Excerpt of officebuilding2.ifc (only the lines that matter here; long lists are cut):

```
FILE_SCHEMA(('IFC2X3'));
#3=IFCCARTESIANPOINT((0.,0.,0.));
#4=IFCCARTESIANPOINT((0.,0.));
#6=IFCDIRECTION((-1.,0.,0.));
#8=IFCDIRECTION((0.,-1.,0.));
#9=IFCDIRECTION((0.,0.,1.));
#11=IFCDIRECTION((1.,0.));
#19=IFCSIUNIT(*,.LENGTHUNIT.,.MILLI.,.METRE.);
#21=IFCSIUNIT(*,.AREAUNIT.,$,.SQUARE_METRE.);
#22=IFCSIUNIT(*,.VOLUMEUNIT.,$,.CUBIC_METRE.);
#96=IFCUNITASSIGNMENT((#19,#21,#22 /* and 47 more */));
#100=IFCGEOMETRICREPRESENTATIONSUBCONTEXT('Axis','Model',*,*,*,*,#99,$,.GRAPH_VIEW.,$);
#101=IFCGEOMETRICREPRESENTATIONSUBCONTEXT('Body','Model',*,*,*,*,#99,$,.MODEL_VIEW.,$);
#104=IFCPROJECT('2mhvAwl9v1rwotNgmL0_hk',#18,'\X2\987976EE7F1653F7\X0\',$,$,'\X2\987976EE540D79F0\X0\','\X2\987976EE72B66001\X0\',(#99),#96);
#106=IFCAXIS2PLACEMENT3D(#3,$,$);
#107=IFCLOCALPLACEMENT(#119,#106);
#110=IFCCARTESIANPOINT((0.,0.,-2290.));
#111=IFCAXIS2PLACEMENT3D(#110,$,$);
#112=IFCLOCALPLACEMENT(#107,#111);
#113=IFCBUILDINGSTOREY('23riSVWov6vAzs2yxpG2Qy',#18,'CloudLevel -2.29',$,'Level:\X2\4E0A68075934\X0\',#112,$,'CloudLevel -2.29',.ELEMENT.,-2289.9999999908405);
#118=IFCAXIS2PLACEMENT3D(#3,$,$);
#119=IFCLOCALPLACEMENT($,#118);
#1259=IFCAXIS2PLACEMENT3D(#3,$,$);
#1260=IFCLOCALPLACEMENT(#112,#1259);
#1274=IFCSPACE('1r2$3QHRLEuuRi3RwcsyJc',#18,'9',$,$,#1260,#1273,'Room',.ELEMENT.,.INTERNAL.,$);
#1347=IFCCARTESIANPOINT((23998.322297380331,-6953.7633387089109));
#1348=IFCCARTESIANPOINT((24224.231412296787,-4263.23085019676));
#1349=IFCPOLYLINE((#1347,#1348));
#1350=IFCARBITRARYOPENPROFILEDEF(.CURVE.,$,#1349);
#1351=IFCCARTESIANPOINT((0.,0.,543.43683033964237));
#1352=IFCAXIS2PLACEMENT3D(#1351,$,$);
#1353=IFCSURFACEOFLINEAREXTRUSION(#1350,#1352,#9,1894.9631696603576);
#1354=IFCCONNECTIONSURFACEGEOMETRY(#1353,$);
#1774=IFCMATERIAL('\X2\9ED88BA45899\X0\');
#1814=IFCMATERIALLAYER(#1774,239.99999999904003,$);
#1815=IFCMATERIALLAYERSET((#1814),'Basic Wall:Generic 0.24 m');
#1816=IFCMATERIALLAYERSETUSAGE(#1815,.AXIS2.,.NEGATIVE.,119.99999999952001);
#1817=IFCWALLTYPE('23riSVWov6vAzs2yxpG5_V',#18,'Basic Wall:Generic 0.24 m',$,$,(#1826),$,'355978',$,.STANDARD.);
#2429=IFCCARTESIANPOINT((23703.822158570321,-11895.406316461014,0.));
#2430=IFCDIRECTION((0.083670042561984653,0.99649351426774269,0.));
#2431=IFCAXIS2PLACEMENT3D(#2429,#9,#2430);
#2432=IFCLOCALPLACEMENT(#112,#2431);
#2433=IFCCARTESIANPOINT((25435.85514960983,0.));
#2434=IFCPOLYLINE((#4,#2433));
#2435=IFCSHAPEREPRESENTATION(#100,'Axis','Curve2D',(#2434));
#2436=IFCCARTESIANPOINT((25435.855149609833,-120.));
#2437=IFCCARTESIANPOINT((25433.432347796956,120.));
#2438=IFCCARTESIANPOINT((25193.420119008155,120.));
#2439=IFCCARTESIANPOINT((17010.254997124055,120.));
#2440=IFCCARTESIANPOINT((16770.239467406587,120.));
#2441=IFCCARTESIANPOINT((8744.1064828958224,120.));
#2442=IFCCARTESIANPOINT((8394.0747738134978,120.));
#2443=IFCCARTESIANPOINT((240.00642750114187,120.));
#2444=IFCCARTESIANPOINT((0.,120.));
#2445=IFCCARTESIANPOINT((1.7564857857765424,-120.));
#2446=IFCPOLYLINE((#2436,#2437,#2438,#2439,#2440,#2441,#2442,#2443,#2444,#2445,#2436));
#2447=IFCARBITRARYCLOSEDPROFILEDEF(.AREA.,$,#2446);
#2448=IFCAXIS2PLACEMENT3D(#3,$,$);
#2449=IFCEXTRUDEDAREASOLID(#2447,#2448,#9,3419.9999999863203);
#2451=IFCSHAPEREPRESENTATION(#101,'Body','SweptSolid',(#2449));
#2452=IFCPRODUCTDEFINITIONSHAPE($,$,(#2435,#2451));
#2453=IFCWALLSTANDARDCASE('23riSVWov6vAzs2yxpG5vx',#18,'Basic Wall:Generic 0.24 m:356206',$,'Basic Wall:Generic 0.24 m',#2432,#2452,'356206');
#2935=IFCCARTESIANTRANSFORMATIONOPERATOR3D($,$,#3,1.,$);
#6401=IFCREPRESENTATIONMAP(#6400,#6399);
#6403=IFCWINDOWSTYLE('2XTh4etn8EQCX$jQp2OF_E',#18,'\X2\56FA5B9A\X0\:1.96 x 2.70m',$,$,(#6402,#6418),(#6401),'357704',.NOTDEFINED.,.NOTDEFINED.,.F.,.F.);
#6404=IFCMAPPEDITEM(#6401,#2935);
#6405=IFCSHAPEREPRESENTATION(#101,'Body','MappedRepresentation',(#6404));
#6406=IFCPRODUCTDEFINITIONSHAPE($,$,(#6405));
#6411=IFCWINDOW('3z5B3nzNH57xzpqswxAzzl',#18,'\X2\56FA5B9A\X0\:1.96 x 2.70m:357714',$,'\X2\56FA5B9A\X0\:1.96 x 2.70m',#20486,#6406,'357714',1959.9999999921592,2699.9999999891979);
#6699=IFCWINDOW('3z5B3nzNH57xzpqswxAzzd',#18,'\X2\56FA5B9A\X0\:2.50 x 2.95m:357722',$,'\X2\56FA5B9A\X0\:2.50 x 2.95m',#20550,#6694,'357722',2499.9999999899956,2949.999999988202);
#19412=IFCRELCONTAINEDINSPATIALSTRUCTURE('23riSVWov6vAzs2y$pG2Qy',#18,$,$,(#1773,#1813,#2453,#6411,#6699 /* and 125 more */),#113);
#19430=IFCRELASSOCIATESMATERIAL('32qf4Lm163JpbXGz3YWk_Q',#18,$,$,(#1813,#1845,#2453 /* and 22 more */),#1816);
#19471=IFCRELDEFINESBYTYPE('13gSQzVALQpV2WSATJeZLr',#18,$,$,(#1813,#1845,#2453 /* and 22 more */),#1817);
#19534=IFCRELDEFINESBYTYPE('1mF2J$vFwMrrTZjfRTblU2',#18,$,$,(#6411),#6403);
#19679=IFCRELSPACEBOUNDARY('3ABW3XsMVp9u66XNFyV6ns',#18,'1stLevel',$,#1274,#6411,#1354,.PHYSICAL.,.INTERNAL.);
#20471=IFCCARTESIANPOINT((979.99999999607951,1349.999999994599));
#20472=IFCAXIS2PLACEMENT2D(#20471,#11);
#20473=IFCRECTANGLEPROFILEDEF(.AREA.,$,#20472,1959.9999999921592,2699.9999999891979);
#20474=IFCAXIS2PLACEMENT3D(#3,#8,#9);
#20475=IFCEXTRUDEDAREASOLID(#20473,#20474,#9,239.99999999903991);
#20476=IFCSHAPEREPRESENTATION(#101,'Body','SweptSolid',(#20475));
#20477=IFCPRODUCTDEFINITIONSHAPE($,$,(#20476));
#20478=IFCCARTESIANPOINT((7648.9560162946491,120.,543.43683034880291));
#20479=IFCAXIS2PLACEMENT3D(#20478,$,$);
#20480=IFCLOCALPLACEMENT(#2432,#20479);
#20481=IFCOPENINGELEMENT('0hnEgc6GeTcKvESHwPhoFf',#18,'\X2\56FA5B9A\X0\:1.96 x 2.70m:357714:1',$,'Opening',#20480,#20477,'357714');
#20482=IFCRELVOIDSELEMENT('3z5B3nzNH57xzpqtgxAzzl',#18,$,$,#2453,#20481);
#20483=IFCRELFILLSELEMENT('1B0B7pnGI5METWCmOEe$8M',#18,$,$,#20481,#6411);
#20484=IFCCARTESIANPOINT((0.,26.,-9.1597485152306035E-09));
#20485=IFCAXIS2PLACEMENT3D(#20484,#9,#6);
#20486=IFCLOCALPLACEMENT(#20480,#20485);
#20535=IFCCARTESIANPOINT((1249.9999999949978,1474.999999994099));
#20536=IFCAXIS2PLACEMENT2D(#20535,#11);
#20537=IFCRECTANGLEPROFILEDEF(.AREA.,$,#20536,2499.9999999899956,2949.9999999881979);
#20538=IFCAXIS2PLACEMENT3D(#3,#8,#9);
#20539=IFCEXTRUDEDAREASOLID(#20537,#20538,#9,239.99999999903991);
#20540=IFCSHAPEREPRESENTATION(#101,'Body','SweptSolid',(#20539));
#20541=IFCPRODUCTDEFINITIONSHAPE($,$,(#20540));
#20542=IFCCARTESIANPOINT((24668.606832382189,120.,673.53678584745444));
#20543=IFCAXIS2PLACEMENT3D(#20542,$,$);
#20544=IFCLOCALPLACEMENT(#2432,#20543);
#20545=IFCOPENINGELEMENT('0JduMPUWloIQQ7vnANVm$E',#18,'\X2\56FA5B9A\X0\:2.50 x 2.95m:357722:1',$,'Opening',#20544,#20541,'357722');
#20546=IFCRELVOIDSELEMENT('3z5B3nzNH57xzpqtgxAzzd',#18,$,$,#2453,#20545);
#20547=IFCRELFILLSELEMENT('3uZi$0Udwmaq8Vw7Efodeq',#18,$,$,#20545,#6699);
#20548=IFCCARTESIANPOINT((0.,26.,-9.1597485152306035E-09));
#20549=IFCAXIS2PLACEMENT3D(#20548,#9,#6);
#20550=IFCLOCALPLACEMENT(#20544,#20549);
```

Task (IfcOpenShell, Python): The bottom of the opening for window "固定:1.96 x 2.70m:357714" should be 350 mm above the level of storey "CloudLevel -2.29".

```python
import numpy as np
import ifcopenshell
import ifcopenshell.api.geometry
import ifcopenshell.geom
import ifcopenshell.util.element
import ifcopenshell.util.placement
import ifcopenshell.util.shape
import ifcopenshell.util.unit

model = ifcopenshell.open("officebuilding2.ifc")
unit_scale = ifcopenshell.util.unit.calculate_unit_scale(model)

window = model.by_id(6411)
opening = window.FillsVoids[0].RelatingOpeningElement
storey = ifcopenshell.util.element.get_container(window, ifc_class="IfcBuildingStorey")
level = ifcopenshell.util.placement.get_local_placement(storey.ObjectPlacement)[2, 3]

# The opening's origin need not be at the sill, so measure its lowest point.
shape = ifcopenshell.geom.create_shape(ifcopenshell.geom.settings(), opening)
bottom = ifcopenshell.util.shape.get_shape_bottom_elevation(shape, shape.geometry) / unit_scale
dz = level + 0.35 / unit_scale - bottom

shift = np.array([0.0, 0.0, dz])
# The window is placed relative to its opening, so it follows when the opening moves.
matrix = ifcopenshell.util.placement.get_local_placement(opening.ObjectPlacement)
matrix[:3, 3] += shift
ifcopenshell.api.geometry.edit_object_placement(
    model, product=opening, matrix=matrix, is_si=False, should_transform_children=True
)

# Space boundary surfaces are stored in each space's coordinates; move them too.
for rel in window.ProvidesBoundaries:
    if not rel.ConnectionGeometry:
        continue
    surface = rel.ConnectionGeometry.SurfaceOnRelatingElement
    space_matrix = ifcopenshell.util.placement.get_local_placement(rel.RelatingSpace.ObjectPlacement)
    point = np.array(surface.Position.Location.Coordinates) + space_matrix[:3, :3].T @ shift
    surface.Position = model.createIfcAxis2Placement3D(
        model.createIfcCartesianPoint(point.tolist()), surface.Position.Axis, surface.Position.RefDirection
    )

print(f"moved by {dz * unit_scale:+.3f} m")

model.write("officebuilding2_updated.ifc")
```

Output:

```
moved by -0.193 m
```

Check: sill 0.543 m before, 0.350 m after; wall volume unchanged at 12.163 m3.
